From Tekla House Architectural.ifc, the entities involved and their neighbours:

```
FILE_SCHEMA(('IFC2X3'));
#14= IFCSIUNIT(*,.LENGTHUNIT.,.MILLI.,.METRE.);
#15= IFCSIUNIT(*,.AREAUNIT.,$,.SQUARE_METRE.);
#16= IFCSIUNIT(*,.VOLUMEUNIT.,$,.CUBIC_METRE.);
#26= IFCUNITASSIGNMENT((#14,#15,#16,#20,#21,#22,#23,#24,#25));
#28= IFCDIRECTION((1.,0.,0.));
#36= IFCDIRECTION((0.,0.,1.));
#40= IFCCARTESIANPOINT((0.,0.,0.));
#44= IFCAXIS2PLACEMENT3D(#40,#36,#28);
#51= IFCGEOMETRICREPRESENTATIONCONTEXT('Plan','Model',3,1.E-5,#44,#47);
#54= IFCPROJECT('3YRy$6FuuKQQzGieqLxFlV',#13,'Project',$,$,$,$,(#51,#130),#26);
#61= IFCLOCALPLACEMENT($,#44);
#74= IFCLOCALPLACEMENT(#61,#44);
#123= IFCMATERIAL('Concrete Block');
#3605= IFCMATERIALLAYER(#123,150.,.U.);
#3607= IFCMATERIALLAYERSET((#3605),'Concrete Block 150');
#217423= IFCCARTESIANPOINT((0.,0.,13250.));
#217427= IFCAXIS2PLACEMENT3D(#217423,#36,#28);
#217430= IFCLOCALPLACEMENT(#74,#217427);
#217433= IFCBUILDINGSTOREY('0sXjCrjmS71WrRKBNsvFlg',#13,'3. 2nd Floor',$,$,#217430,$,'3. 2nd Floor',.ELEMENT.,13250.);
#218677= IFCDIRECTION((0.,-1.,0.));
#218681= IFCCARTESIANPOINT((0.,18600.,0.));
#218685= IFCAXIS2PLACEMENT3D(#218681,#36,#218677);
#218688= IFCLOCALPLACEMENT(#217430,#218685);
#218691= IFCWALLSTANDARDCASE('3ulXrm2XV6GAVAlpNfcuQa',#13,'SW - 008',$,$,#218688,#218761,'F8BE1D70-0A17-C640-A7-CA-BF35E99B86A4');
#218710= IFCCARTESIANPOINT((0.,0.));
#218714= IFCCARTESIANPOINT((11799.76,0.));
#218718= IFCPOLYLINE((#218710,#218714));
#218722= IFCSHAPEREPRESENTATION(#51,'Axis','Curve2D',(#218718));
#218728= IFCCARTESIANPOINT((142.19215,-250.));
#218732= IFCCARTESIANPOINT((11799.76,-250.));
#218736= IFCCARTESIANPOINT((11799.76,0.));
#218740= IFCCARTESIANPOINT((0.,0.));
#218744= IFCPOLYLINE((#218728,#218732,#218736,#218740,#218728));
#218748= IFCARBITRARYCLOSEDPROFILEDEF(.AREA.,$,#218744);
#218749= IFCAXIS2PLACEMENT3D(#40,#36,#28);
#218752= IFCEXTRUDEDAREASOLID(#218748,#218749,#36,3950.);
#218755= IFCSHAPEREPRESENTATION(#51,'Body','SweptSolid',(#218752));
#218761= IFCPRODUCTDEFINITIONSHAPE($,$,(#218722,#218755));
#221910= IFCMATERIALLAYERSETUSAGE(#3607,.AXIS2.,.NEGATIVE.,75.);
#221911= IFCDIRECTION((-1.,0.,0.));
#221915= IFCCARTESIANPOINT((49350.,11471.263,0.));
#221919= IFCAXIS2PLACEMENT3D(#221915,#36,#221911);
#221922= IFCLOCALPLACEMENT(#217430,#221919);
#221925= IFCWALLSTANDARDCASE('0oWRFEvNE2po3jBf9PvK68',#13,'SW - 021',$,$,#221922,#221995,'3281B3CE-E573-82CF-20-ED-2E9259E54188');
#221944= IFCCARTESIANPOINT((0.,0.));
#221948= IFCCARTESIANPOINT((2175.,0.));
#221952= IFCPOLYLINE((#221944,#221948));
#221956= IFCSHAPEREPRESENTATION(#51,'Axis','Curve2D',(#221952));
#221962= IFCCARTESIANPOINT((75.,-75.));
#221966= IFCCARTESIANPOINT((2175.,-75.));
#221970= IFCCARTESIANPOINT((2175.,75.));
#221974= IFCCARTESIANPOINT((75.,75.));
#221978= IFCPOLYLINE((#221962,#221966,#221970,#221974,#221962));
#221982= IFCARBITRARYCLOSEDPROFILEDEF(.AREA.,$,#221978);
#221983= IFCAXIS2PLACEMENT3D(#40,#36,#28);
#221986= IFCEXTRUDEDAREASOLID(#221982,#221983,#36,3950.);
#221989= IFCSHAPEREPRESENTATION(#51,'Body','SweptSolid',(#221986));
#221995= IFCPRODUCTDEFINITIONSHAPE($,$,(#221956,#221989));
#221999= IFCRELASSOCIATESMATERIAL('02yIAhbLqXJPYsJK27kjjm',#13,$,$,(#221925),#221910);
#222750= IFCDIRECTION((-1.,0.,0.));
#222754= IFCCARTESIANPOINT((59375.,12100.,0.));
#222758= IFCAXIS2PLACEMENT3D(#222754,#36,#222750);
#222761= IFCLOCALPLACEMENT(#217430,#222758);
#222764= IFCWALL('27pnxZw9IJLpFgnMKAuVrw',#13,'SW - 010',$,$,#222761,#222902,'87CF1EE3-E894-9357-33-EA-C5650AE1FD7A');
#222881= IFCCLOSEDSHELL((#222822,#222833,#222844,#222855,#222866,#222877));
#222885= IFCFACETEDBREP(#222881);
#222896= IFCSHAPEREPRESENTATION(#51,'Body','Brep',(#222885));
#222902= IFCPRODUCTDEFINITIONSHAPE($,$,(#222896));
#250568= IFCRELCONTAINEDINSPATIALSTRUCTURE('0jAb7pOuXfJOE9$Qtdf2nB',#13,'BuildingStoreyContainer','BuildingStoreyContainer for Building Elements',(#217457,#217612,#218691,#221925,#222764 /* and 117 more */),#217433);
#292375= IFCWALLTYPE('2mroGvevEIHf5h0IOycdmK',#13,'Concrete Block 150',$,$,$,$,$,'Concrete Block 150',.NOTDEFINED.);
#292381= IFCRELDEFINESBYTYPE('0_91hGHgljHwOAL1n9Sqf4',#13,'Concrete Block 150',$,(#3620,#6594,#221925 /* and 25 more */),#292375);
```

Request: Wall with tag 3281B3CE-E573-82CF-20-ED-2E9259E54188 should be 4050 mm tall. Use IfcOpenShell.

```python
import ifcopenshell
import ifcopenshell.geom
import ifcopenshell.util.shape

model = ifcopenshell.open("Tekla House Architectural.ifc")
settings = ifcopenshell.geom.settings()


def volume(element):
    """Net volume in cubic metres, openings subtracted."""
    shape = ifcopenshell.geom.create_shape(settings, element)
    return ifcopenshell.util.shape.get_volume(shape.geometry)


wall = model.by_guid("0oWRFEvNE2po3jBf9PvK68")
before = volume(wall)

body = next(r for r in wall.Representation.Representations if r.RepresentationIdentifier == "Body")
solid = body.Items[0]
old_height = solid.Depth
solid.Depth = 4050.0
after = volume(wall)

print(f"height {old_height:g} -> {solid.Depth:g}, volume {before:.3f} -> {after:.3f} m3")

model.write("Tekla House Architectural_rev.ifc")
```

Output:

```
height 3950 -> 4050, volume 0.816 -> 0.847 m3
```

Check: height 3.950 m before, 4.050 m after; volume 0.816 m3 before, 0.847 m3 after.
